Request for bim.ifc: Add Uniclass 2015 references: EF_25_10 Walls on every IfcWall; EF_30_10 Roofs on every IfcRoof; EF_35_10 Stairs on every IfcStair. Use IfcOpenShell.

First a look at what the model holds.

```python
import ifcopenshell

model = ifcopenshell.open("bim.ifc")
print(model.schema)
print("classifications:", [c.Name for c in model.by_type("IfcClassification")])
for ifc_class in ("IfcDoor", "IfcRoof", "IfcStair", "IfcWall", "IfcWindow"):
    print(ifc_class, len(model.by_type(ifc_class)))
```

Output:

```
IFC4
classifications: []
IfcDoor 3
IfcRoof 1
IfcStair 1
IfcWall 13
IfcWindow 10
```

```python
import ifcopenshell
import ifcopenshell.api.classification

model = ifcopenshell.open("bim.ifc")

system = ifcopenshell.api.classification.add_classification(model, classification="Uniclass 2015")

codes = {
    "IfcWall": ("EF_25_10", "Walls"),
    "IfcRoof": ("EF_30_10", "Roofs"),
    "IfcStair": ("EF_35_10", "Stairs"),
}
for ifc_class, (code, name) in codes.items():
    products = model.by_type(ifc_class)
    ifcopenshell.api.classification.add_reference(
        model, products=products, classification=system, identification=code, name=name
    )
    print(code, len(products))

model.write("bim_updated.ifc")
```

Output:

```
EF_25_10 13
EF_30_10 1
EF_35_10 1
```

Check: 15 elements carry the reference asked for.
